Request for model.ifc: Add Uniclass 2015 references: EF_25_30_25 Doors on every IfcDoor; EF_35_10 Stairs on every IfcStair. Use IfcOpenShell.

First a look at what the model holds.

```python
import ifcopenshell

model = ifcopenshell.open("model.ifc")
print(model.schema)
print("classifications:", [c.Name for c in model.by_type("IfcClassification")])
for ifc_class in ("IfcDoor", "IfcRoof", "IfcStair", "IfcWall", "IfcWindow"):
    print(ifc_class, len(model.by_type(ifc_class)))
```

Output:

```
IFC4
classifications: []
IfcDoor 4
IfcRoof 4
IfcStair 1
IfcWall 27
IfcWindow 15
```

```python
import ifcopenshell
import ifcopenshell.api.classification

model = ifcopenshell.open("model.ifc")

system = ifcopenshell.api.classification.add_classification(model, classification="Uniclass 2015")

codes = {
    "IfcDoor": ("EF_25_30_25", "Doors"),
    "IfcStair": ("EF_35_10", "Stairs"),
}
for ifc_class, (code, name) in codes.items():
    products = model.by_type(ifc_class)
    ifcopenshell.api.classification.add_reference(
        model, products=products, classification=system, identification=code, name=name
    )
    print(code, len(products))

model.write("model_edited.ifc")
```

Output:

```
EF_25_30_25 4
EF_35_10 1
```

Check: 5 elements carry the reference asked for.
